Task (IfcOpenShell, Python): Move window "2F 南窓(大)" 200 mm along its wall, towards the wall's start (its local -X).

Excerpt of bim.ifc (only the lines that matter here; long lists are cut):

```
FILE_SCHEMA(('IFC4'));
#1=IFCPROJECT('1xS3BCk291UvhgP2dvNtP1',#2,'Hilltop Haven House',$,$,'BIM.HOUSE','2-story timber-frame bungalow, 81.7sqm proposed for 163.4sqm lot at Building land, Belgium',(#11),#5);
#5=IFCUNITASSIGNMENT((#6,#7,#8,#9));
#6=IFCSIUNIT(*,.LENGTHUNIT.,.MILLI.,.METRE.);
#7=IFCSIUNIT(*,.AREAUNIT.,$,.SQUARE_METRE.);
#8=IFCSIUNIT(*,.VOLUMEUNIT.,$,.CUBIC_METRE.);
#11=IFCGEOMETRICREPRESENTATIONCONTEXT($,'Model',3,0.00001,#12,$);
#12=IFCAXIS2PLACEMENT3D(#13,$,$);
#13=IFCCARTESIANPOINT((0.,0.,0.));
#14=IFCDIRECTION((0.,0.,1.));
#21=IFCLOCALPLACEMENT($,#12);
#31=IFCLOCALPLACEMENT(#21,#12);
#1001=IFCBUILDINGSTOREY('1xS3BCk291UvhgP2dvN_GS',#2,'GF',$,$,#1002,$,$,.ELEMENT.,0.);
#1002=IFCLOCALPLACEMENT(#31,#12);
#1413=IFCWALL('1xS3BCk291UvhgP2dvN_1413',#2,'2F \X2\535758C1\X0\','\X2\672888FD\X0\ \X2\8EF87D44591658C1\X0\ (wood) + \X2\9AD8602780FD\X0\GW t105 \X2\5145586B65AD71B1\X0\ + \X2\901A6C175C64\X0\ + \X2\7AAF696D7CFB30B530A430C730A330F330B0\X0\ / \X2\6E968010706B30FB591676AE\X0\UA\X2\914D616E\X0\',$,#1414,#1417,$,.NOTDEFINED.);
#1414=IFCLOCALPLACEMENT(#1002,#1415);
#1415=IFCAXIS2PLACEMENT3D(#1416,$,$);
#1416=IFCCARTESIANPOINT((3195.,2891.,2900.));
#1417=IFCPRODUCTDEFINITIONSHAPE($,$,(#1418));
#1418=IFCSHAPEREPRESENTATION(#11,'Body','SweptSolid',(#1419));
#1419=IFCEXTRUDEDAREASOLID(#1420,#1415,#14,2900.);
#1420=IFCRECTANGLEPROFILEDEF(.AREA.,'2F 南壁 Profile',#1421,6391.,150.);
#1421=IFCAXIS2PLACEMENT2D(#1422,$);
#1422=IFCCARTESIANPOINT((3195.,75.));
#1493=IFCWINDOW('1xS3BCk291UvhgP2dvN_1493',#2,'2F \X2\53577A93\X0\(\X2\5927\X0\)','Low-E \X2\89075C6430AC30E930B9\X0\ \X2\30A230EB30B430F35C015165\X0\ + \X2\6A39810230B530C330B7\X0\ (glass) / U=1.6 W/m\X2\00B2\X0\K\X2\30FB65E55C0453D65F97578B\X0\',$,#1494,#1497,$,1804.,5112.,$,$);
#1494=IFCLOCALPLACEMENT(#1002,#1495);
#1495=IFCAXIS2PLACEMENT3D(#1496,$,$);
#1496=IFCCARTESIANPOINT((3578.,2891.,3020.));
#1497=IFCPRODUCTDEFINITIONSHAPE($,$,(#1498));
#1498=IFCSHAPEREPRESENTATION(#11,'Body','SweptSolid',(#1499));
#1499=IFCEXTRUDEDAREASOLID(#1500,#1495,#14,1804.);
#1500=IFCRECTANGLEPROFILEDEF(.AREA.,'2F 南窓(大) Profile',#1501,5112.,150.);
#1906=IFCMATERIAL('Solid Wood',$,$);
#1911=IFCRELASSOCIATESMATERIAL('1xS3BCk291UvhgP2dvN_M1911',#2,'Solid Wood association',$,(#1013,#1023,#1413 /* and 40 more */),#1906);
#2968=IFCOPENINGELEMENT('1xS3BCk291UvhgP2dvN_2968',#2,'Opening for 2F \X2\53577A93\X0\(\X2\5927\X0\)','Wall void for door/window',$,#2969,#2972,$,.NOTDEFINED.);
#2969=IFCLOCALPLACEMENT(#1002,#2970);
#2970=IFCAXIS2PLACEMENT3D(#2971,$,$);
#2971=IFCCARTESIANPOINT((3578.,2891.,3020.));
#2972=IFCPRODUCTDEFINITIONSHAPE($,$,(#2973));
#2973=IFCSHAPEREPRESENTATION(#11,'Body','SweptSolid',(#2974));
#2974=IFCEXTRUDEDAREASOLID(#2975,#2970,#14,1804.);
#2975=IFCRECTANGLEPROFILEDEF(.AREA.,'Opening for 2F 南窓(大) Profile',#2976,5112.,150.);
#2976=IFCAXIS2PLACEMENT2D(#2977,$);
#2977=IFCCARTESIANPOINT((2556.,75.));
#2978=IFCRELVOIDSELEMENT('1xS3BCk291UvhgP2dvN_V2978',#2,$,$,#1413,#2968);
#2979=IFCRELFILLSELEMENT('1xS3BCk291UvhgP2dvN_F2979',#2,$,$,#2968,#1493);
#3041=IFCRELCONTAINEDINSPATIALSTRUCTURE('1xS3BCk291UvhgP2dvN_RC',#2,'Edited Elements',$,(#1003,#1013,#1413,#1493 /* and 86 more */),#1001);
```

```python
import ifcopenshell
import ifcopenshell.api.geometry
import ifcopenshell.util.placement
import ifcopenshell.util.unit

model = ifcopenshell.open("bim.ifc")
unit_scale = ifcopenshell.util.unit.calculate_unit_scale(model)

window = model.by_guid("1xS3BCk291UvhgP2dvN_1493")
opening = window.FillsVoids[0].RelatingOpeningElement
wall = opening.VoidsElements[0].RelatingBuildingElement

wall_matrix = ifcopenshell.util.placement.get_local_placement(wall.ObjectPlacement)
shift = wall_matrix[:3, 0] * -0.2 / unit_scale
before = ifcopenshell.util.placement.get_local_placement(window.ObjectPlacement)[:3, 3].copy()

# The window is not placed relative to its opening, so move both.
for product in (opening, window):
    matrix = ifcopenshell.util.placement.get_local_placement(product.ObjectPlacement)
    matrix[:3, 3] += shift
    ifcopenshell.api.geometry.edit_object_placement(model, product=product, matrix=matrix, is_si=False)

after = ifcopenshell.util.placement.get_local_placement(window.ObjectPlacement)[:3, 3]
print("window moved by", (after - before).round(3) + 0.0)

model.write("bim_rev.ifc")
```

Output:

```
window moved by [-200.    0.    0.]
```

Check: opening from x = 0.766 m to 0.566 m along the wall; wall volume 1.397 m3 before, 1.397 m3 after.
